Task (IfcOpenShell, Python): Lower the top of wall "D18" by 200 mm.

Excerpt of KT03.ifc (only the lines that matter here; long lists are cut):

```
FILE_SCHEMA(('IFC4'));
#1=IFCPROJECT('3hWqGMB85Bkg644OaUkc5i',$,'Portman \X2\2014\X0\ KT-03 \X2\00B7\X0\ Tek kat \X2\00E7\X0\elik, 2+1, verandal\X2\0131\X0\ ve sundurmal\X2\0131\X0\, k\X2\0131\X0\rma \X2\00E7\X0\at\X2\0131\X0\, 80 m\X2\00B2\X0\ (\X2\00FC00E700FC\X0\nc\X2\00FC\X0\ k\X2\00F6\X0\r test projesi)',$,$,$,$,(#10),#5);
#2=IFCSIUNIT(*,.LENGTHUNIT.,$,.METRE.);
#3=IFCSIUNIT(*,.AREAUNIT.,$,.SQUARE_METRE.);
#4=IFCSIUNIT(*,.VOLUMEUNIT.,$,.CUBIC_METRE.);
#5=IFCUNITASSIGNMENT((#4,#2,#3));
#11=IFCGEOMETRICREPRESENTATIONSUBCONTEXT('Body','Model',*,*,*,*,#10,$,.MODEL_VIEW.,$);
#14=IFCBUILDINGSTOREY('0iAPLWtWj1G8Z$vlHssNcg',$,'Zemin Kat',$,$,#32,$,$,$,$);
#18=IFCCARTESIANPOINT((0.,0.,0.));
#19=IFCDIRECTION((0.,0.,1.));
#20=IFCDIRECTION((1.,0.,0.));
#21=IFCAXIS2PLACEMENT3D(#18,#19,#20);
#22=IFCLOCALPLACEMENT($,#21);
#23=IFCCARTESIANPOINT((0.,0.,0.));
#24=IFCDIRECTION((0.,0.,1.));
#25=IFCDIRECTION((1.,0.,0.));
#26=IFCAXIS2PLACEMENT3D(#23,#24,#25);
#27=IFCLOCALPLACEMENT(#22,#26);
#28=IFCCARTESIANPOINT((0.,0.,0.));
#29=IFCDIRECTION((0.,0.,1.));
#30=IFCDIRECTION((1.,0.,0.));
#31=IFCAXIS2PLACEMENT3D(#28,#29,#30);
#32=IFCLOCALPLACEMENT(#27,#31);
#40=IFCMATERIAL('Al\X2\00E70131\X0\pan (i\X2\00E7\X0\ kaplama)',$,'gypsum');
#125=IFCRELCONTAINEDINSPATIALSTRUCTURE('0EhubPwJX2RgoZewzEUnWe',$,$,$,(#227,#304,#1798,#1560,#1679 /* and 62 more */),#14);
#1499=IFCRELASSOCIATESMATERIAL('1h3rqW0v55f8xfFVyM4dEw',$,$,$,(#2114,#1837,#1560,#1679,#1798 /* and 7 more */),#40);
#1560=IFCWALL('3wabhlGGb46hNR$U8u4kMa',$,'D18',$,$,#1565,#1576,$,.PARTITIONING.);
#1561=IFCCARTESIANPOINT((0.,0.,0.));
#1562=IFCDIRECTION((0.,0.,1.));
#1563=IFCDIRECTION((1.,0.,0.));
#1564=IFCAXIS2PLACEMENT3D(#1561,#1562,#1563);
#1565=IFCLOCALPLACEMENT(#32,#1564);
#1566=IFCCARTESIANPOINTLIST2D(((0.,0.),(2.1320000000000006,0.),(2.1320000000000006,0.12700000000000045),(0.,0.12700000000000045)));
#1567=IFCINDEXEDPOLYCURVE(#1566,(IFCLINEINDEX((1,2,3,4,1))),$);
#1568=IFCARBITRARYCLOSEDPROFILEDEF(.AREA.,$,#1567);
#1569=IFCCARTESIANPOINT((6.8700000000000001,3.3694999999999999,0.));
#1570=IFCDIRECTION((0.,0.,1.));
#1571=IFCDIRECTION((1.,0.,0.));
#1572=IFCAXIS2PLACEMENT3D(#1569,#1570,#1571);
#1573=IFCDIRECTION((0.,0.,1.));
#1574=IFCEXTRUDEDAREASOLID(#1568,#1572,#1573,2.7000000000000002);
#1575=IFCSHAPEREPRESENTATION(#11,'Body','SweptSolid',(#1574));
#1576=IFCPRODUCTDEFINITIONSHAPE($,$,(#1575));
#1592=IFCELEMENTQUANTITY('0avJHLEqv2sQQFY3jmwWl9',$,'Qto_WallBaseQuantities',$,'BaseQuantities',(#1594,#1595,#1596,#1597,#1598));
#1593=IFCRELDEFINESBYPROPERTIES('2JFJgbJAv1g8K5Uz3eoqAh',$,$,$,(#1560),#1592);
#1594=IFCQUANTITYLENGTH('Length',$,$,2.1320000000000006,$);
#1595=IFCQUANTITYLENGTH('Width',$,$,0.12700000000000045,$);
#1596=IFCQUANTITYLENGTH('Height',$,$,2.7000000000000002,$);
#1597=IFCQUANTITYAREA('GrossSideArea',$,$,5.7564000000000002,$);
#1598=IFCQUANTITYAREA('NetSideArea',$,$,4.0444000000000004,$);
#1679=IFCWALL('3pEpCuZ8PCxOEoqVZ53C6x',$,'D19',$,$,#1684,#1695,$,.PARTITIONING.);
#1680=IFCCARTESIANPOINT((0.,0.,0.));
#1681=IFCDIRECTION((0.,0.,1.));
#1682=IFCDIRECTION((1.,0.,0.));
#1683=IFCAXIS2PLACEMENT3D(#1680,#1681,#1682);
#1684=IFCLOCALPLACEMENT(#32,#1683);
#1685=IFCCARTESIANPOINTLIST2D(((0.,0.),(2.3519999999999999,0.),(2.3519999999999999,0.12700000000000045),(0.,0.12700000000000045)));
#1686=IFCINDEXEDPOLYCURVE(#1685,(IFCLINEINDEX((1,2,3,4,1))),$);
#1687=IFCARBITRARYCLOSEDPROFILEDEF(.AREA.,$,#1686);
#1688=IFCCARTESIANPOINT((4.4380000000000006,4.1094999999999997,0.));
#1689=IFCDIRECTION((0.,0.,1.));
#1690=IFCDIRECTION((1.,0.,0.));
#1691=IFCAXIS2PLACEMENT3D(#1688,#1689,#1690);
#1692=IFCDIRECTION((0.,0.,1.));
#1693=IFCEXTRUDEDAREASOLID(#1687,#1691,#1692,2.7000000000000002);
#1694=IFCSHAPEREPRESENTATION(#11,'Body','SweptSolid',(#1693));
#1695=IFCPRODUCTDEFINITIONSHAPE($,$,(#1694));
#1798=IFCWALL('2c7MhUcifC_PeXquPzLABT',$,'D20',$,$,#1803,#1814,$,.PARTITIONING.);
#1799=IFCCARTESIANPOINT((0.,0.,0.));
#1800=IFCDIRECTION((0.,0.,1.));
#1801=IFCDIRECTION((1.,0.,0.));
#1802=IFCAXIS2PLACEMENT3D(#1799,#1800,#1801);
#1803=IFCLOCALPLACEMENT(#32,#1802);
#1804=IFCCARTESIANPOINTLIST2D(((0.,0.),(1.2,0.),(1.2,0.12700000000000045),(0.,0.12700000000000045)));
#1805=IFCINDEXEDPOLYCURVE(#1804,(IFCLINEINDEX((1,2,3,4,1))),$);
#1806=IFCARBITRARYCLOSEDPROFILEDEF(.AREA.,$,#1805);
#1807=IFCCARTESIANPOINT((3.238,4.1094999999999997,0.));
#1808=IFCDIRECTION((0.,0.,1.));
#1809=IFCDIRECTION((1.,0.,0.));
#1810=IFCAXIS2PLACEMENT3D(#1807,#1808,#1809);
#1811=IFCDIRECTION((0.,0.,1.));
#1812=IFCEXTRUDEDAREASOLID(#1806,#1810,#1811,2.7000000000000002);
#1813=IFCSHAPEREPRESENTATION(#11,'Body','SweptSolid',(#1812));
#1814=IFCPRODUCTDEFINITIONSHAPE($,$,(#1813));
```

```python
import ifcopenshell
import ifcopenshell.api.pset
import ifcopenshell.geom
import ifcopenshell.util.element
import ifcopenshell.util.representation
import ifcopenshell.util.shape
import ifcopenshell.util.unit

model = ifcopenshell.open("KT03.ifc")
unit_scale = ifcopenshell.util.unit.calculate_unit_scale(model)
area_scale = ifcopenshell.util.unit.calculate_unit_scale(model, "AREAUNIT")
settings = ifcopenshell.geom.settings()


def volume(element):
    """Net volume in cubic metres, openings subtracted."""
    shape = ifcopenshell.geom.create_shape(settings, element)
    return ifcopenshell.util.shape.get_volume(shape.geometry)


wall = model.by_guid("3wabhlGGb46hNR$U8u4kMa")
before = volume(wall)

body = ifcopenshell.util.representation.get_representation(wall, "Model", "Body")
solid = body.Items[0]
old_height = solid.Depth
solid.Depth -= 0.2 / unit_scale
after = volume(wall)
thickness = 0.127  # wall thickness in metres

# Update the stored height, areas and volumes.
qto = model.by_id(ifcopenshell.util.element.get_pset(wall, "Qto_WallBaseQuantities", should_inherit=False)["id"])
ifcopenshell.api.pset.edit_qto(model, qto=qto, properties={
    "Height": solid.Depth,
    "GrossSideArea": ifcopenshell.util.element.get_pset(wall, "Qto_WallBaseQuantities", "GrossSideArea") * solid.Depth / old_height,
    "NetSideArea": after / thickness / area_scale,
})

print(f"height {old_height:g} -> {solid.Depth:g}, volume {before:.3f} -> {after:.3f} m3")

model.write("KT03_v2.ifc")
```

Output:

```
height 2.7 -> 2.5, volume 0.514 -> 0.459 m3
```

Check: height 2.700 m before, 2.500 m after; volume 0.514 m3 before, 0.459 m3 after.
